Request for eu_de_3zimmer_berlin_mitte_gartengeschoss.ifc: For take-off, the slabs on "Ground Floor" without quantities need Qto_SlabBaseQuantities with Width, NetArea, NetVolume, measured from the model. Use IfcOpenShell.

First a look at what the model holds.

```python
import ifcopenshell
import ifcopenshell.util.element
import ifcopenshell.util.unit

model = ifcopenshell.open("eu_de_3zimmer_berlin_mitte_gartengeschoss.ifc")
print(model.schema)
for unit_type in ("LENGTHUNIT", "AREAUNIT", "VOLUMEUNIT"):
    print(unit_type, ifcopenshell.util.unit.calculate_unit_scale(model, unit_type))
storey = next(s for s in model.by_type("IfcBuildingStorey") if s.Name == "Ground Floor")
slabs = [e for e in ifcopenshell.util.element.get_decomposition(storey) if e.is_a("IfcSlab")]
for e in sorted(slabs, key=lambda e: e.id()):
    print(e.id(), e.is_a(), e.Name, list(ifcopenshell.util.element.get_psets(e, qtos_only=True)), sep=" | ")
```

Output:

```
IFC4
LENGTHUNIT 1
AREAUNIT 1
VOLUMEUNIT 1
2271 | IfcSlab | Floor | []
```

```python
import ifcopenshell
import ifcopenshell.api.pset
import ifcopenshell.geom
import ifcopenshell.util.element
import ifcopenshell.util.shape
import ifcopenshell.util.unit

model = ifcopenshell.open("eu_de_3zimmer_berlin_mitte_gartengeschoss.ifc")
unit_scale = ifcopenshell.util.unit.calculate_unit_scale(model)
area_scale = ifcopenshell.util.unit.calculate_unit_scale(model, "AREAUNIT")
volume_scale = ifcopenshell.util.unit.calculate_unit_scale(model, "VOLUMEUNIT")
settings = ifcopenshell.geom.settings()

storey = next(s for s in model.by_type("IfcBuildingStorey") if s.Name == "Ground Floor")
slabs = [e for e in ifcopenshell.util.element.get_decomposition(storey) if e.is_a("IfcSlab")]

for e in sorted(slabs, key=lambda e: e.id()):
    if ifcopenshell.util.element.get_psets(e, qtos_only=True, should_inherit=False):
        continue
    # Geometry comes back in metres, in the element's own axes.
    shape = ifcopenshell.geom.create_shape(settings, e)
    values = {
        "Width": ifcopenshell.util.shape.get_z(shape.geometry) / unit_scale,
        "NetArea": ifcopenshell.util.shape.get_footprint_area(shape.geometry) / area_scale,
        "NetVolume": ifcopenshell.util.shape.get_volume(shape.geometry) / volume_scale,
    }
    qto = ifcopenshell.api.pset.add_qto(model, product=e, name="Qto_SlabBaseQuantities")
    ifcopenshell.api.pset.edit_qto(model, qto=qto, properties=values)
    print(e.id(), {k: round(v, 3) for k, v in values.items()})

model.write("eu_de_3zimmer_berlin_mitte_gartengeschoss_edited.ifc")
```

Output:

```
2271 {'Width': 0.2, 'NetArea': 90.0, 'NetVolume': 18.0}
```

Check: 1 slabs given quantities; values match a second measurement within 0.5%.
